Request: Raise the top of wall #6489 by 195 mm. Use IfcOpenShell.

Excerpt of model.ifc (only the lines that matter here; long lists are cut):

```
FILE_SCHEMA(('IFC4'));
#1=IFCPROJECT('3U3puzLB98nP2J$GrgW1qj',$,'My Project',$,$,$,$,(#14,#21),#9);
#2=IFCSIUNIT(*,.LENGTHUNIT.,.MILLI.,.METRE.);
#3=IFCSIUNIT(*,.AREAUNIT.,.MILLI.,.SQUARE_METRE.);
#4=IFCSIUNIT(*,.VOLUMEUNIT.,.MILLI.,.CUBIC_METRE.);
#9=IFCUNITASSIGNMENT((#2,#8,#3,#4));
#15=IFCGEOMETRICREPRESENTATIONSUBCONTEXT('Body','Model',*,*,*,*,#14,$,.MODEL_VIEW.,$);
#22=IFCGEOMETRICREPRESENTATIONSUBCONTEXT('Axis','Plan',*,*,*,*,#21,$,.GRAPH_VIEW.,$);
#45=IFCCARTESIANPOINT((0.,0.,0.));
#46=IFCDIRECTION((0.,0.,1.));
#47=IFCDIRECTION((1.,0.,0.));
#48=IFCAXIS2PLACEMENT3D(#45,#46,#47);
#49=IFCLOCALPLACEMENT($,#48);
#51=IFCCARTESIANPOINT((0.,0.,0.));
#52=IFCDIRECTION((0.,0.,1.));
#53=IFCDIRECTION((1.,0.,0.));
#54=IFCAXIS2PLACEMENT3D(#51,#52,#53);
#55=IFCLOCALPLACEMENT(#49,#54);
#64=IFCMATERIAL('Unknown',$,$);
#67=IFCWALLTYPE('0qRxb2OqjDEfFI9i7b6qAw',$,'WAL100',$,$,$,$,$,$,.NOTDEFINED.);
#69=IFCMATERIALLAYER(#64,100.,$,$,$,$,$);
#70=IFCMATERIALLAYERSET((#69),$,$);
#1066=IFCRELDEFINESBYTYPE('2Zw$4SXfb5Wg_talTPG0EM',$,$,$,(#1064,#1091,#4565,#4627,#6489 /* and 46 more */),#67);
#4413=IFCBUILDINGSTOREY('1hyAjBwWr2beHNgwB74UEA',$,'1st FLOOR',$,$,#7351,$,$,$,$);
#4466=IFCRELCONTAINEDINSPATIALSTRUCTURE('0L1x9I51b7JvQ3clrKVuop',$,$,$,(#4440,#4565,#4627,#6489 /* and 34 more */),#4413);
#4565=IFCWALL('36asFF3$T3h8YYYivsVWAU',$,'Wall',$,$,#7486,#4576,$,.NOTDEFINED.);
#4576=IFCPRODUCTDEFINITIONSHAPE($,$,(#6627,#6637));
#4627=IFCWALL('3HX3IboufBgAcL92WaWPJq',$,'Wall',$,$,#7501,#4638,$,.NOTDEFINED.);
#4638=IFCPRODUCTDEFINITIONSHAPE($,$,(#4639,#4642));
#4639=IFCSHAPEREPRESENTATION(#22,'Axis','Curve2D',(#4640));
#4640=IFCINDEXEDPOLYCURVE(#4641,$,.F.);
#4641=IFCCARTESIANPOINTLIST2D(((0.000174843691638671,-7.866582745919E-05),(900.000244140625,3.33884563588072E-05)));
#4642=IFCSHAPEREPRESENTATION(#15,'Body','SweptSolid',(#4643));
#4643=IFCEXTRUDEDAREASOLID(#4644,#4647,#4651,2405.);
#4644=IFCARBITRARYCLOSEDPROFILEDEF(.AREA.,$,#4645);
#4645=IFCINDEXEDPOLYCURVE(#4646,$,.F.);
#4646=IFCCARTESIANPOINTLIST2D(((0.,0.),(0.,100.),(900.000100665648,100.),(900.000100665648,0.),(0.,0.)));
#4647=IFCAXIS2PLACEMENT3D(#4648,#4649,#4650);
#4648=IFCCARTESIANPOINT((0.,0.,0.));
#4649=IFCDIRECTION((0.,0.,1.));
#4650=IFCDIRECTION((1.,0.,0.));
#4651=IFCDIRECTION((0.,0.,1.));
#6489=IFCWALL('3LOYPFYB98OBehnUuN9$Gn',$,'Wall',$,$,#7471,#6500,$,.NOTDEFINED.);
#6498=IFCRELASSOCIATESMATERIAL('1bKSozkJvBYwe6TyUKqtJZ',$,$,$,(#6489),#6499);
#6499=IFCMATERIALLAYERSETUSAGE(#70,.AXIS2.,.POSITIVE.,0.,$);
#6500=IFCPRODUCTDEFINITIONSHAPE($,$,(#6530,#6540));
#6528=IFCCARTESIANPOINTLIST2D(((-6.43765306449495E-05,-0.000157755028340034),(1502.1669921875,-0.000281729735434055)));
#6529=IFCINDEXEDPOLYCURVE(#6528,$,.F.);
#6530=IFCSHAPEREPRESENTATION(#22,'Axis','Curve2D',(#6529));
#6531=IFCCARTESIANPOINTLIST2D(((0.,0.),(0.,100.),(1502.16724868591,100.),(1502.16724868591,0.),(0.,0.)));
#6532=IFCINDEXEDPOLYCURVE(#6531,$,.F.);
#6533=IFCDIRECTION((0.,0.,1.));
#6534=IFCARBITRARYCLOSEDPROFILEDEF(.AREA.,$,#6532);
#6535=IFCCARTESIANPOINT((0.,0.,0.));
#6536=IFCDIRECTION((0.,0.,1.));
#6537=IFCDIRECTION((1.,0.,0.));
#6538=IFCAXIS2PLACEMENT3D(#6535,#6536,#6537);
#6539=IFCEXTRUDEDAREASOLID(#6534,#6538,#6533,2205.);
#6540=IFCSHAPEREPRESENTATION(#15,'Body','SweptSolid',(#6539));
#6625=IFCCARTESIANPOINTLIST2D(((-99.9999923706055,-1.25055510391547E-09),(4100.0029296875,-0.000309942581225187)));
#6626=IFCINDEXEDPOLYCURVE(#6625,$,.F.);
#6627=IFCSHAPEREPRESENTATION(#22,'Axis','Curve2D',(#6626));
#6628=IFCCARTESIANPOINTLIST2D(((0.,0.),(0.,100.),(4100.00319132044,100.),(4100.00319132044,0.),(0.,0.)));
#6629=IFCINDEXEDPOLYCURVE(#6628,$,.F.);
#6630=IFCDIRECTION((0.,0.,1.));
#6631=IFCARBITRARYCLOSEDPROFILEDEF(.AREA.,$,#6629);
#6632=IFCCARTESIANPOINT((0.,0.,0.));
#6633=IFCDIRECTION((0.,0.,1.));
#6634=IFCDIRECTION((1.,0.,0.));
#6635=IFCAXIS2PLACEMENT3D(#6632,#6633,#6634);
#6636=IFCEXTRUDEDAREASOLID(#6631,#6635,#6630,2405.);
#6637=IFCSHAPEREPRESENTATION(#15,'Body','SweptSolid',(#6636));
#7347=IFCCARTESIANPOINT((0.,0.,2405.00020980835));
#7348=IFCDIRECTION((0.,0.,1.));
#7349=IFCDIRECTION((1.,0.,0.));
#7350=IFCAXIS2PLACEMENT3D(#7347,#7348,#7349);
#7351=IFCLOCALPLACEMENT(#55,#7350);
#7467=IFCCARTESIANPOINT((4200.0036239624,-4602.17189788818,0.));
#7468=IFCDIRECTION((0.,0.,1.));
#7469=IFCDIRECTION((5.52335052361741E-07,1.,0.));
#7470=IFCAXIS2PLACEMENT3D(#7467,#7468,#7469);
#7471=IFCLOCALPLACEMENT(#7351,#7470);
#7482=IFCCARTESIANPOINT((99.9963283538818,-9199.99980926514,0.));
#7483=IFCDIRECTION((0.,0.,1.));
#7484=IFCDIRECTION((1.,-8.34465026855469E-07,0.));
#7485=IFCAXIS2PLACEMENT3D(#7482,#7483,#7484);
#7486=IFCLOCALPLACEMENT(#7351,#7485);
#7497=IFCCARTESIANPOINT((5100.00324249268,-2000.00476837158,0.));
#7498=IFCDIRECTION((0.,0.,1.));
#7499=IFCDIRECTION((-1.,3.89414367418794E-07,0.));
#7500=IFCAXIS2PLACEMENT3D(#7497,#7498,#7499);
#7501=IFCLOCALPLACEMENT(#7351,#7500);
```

```python
import ifcopenshell
import ifcopenshell.geom
import ifcopenshell.util.representation
import ifcopenshell.util.shape
import ifcopenshell.util.unit

model = ifcopenshell.open("model.ifc")
unit_scale = ifcopenshell.util.unit.calculate_unit_scale(model)
settings = ifcopenshell.geom.settings()


def volume(element):
    """Net volume in cubic metres, openings subtracted."""
    shape = ifcopenshell.geom.create_shape(settings, element)
    return ifcopenshell.util.shape.get_volume(shape.geometry)


wall = model.by_guid("3LOYPFYB98OBehnUuN9$Gn")
before = volume(wall)

body = ifcopenshell.util.representation.get_representation(wall, "Model", "Body")
solid = body.Items[0]
old_height = solid.Depth
solid.Depth += 0.195 / unit_scale
after = volume(wall)

print(f"height {old_height:g} -> {solid.Depth:g}, volume {before:.3f} -> {after:.3f} m3")

model.write("model_updated.ifc")
```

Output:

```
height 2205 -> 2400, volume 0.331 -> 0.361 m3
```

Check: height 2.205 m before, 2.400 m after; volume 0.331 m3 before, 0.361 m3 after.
